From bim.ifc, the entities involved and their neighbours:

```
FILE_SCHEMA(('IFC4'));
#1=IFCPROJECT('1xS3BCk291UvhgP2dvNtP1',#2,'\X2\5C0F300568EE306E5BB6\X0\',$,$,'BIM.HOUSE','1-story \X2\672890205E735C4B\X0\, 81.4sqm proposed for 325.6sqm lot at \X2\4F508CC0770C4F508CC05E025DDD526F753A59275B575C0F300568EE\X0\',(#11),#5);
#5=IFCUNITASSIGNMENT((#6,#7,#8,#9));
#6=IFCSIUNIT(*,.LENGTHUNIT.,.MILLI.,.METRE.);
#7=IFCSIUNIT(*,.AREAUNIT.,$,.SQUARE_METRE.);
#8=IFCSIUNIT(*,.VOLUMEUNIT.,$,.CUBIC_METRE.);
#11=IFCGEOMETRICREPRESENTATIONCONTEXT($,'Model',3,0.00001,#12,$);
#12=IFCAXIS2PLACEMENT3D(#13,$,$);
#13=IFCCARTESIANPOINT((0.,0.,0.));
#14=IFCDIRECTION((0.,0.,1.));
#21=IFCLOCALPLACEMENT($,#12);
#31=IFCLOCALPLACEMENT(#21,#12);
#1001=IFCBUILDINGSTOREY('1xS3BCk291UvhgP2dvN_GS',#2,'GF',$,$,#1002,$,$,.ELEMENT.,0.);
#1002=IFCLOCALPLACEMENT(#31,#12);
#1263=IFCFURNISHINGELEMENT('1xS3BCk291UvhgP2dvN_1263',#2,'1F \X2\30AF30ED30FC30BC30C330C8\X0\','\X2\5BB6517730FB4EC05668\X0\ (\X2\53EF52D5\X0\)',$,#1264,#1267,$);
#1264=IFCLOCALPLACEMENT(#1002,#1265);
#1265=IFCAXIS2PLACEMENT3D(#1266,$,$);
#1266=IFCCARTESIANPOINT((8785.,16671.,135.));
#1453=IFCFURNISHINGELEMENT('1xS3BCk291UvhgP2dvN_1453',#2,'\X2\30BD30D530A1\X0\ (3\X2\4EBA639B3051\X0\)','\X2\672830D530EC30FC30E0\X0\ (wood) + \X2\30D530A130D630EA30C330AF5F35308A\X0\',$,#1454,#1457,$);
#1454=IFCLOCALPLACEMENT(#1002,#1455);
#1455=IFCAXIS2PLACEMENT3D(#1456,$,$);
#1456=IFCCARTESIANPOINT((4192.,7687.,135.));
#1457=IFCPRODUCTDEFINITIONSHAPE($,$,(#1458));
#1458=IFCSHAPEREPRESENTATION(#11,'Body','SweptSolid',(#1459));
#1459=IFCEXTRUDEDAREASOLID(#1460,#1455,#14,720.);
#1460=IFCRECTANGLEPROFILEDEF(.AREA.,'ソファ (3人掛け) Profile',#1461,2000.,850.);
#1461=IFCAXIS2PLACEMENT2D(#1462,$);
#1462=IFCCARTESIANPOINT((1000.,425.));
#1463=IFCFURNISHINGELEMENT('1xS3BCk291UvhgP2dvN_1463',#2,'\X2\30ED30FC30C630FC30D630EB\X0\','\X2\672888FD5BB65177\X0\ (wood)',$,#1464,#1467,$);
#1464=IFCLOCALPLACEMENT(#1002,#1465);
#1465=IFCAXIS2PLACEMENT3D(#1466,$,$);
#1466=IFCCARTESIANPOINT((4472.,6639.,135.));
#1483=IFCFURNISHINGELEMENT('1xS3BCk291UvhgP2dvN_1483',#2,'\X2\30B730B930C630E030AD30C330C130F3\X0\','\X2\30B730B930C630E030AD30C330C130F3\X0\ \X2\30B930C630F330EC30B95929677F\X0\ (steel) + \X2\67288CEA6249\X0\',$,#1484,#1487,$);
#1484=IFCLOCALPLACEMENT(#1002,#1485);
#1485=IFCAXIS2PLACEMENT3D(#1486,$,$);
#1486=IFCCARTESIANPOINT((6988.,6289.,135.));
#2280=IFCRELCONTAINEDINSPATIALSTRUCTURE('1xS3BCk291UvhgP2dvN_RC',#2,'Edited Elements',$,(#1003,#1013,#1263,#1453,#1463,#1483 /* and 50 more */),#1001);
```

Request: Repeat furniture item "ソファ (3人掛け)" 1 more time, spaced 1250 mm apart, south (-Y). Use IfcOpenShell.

```python
import numpy as np
import ifcopenshell
import ifcopenshell.api.geometry
import ifcopenshell.api.root
import ifcopenshell.util.element
import ifcopenshell.util.placement

model = ifcopenshell.open("bim.ifc")


def reuse_history(source, copy):
    """copy_class also copies each property set's owner history, people and application; keep the originals."""
    for rel in copy.IsDefinedBy:
        if rel.is_a("IfcRelDefinesByProperties") and (history := rel.RelatingPropertyDefinition.OwnerHistory):
            rel.RelatingPropertyDefinition.OwnerHistory = source.OwnerHistory
            ifcopenshell.util.element.remove_deep2(model, history)


source = model.by_guid("1xS3BCk291UvhgP2dvN_1453")
base = ifcopenshell.util.placement.get_local_placement(source.ObjectPlacement)
step = np.array([0.0, -1.0, 0.0]) * 1250.0

for i in range(1, 2):
    copy = ifcopenshell.api.root.copy_class(model, product=source)
    copy.Representation = ifcopenshell.util.element.copy_deep(
        model, source.Representation, exclude=["IfcGeometricRepresentationContext", "IfcRepresentationMap"]
    )
    reuse_history(source, copy)
    matrix = base.copy()
    matrix[:3, 3] += i * step
    print("added at", matrix[:3, 3].round(3) + 0.0)
    ifcopenshell.api.geometry.edit_object_placement(model, product=copy, matrix=matrix, is_si=False)

model.write("bim_rev.ifc")
```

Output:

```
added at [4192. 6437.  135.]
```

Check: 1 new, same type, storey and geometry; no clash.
